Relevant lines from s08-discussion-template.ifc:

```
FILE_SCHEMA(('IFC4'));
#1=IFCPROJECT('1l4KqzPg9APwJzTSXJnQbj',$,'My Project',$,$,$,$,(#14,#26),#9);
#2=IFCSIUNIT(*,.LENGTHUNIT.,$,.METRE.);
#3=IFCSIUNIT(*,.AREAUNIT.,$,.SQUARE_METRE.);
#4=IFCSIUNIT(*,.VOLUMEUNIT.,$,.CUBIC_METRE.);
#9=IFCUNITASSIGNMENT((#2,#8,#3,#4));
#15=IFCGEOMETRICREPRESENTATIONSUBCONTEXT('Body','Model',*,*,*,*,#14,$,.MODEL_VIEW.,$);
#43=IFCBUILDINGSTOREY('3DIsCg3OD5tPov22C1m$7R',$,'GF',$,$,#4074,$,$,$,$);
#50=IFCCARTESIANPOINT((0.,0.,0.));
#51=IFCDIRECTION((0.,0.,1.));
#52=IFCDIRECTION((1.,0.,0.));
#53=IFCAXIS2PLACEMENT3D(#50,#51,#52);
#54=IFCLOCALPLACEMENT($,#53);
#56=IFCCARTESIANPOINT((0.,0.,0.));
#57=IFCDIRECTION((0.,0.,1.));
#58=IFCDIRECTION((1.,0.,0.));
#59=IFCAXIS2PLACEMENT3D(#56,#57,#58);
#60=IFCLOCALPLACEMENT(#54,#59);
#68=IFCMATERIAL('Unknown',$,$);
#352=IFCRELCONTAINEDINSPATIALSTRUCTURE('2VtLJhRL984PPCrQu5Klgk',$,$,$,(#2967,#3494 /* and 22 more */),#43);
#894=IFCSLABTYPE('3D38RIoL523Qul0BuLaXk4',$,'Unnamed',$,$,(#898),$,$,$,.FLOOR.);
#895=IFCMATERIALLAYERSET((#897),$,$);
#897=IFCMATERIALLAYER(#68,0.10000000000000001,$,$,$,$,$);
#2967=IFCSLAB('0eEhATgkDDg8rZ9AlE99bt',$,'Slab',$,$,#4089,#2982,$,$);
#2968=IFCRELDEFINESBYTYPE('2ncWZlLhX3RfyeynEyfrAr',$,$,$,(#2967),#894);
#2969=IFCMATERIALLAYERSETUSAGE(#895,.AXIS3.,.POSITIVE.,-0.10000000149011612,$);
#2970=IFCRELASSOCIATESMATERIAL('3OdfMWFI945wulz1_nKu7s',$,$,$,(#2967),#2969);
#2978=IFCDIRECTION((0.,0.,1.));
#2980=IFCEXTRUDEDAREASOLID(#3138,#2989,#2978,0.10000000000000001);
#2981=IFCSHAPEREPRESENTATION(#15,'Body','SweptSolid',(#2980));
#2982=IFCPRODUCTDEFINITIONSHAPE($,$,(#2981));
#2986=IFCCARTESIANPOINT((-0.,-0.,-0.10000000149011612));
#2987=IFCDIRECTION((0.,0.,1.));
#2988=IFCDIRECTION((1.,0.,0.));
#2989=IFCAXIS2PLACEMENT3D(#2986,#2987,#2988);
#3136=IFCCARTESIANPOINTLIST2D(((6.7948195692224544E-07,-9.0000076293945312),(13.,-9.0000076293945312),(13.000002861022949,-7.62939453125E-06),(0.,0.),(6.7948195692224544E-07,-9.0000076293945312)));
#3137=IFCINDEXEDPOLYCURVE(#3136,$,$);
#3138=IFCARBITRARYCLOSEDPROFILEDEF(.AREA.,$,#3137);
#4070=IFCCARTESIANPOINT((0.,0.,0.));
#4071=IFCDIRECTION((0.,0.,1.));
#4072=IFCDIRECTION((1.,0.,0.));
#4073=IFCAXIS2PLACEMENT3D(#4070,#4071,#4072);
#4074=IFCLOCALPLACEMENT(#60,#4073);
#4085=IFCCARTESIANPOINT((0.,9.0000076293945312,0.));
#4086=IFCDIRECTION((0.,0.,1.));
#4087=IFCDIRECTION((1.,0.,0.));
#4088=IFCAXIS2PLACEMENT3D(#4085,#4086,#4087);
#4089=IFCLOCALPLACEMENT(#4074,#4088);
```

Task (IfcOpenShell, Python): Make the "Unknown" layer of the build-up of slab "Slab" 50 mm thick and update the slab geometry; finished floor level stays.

```python
import ifcopenshell
import ifcopenshell.util.element
import ifcopenshell.util.representation
import ifcopenshell.util.unit

model = ifcopenshell.open("s08-discussion-template.ifc")
unit_scale = ifcopenshell.util.unit.calculate_unit_scale(model)

layer_set = model.by_id(895)
layer = next(l for l in layer_set.MaterialLayers if l.Material and l.Material.Name == "Unknown")
change = 0.05 / unit_scale - layer.LayerThickness
layer.LayerThickness += change

# Geometry does not follow the layer set by itself.
slabs = [e for e in ifcopenshell.util.element.get_elements_by_material(model, layer_set) if e.is_a("IfcSlab")]
for slab in sorted(slabs, key=lambda e: e.id()):
    body = ifcopenshell.util.representation.get_representation(slab, "Model", "Body")
    solid = body.Items[0]
    old_depth = solid.Depth
    solid.Depth += change
    # Extruded upwards: lower the start of the extrusion so the top stays.
    x, y, z = solid.Position.Location.Coordinates
    solid.Position.Location = model.createIfcCartesianPoint((x, y, z - change))
    print(slab.id(), f"{old_depth:g} -> {solid.Depth:g}")

# The layers are counted up from the underside, which has moved.
for usage in {ifcopenshell.util.element.get_material(slab) for slab in slabs}:
    usage.OffsetFromReferenceLine -= change

model.write("s08-discussion-template_v2.ifc")
```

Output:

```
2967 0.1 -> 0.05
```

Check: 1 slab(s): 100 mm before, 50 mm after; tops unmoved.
